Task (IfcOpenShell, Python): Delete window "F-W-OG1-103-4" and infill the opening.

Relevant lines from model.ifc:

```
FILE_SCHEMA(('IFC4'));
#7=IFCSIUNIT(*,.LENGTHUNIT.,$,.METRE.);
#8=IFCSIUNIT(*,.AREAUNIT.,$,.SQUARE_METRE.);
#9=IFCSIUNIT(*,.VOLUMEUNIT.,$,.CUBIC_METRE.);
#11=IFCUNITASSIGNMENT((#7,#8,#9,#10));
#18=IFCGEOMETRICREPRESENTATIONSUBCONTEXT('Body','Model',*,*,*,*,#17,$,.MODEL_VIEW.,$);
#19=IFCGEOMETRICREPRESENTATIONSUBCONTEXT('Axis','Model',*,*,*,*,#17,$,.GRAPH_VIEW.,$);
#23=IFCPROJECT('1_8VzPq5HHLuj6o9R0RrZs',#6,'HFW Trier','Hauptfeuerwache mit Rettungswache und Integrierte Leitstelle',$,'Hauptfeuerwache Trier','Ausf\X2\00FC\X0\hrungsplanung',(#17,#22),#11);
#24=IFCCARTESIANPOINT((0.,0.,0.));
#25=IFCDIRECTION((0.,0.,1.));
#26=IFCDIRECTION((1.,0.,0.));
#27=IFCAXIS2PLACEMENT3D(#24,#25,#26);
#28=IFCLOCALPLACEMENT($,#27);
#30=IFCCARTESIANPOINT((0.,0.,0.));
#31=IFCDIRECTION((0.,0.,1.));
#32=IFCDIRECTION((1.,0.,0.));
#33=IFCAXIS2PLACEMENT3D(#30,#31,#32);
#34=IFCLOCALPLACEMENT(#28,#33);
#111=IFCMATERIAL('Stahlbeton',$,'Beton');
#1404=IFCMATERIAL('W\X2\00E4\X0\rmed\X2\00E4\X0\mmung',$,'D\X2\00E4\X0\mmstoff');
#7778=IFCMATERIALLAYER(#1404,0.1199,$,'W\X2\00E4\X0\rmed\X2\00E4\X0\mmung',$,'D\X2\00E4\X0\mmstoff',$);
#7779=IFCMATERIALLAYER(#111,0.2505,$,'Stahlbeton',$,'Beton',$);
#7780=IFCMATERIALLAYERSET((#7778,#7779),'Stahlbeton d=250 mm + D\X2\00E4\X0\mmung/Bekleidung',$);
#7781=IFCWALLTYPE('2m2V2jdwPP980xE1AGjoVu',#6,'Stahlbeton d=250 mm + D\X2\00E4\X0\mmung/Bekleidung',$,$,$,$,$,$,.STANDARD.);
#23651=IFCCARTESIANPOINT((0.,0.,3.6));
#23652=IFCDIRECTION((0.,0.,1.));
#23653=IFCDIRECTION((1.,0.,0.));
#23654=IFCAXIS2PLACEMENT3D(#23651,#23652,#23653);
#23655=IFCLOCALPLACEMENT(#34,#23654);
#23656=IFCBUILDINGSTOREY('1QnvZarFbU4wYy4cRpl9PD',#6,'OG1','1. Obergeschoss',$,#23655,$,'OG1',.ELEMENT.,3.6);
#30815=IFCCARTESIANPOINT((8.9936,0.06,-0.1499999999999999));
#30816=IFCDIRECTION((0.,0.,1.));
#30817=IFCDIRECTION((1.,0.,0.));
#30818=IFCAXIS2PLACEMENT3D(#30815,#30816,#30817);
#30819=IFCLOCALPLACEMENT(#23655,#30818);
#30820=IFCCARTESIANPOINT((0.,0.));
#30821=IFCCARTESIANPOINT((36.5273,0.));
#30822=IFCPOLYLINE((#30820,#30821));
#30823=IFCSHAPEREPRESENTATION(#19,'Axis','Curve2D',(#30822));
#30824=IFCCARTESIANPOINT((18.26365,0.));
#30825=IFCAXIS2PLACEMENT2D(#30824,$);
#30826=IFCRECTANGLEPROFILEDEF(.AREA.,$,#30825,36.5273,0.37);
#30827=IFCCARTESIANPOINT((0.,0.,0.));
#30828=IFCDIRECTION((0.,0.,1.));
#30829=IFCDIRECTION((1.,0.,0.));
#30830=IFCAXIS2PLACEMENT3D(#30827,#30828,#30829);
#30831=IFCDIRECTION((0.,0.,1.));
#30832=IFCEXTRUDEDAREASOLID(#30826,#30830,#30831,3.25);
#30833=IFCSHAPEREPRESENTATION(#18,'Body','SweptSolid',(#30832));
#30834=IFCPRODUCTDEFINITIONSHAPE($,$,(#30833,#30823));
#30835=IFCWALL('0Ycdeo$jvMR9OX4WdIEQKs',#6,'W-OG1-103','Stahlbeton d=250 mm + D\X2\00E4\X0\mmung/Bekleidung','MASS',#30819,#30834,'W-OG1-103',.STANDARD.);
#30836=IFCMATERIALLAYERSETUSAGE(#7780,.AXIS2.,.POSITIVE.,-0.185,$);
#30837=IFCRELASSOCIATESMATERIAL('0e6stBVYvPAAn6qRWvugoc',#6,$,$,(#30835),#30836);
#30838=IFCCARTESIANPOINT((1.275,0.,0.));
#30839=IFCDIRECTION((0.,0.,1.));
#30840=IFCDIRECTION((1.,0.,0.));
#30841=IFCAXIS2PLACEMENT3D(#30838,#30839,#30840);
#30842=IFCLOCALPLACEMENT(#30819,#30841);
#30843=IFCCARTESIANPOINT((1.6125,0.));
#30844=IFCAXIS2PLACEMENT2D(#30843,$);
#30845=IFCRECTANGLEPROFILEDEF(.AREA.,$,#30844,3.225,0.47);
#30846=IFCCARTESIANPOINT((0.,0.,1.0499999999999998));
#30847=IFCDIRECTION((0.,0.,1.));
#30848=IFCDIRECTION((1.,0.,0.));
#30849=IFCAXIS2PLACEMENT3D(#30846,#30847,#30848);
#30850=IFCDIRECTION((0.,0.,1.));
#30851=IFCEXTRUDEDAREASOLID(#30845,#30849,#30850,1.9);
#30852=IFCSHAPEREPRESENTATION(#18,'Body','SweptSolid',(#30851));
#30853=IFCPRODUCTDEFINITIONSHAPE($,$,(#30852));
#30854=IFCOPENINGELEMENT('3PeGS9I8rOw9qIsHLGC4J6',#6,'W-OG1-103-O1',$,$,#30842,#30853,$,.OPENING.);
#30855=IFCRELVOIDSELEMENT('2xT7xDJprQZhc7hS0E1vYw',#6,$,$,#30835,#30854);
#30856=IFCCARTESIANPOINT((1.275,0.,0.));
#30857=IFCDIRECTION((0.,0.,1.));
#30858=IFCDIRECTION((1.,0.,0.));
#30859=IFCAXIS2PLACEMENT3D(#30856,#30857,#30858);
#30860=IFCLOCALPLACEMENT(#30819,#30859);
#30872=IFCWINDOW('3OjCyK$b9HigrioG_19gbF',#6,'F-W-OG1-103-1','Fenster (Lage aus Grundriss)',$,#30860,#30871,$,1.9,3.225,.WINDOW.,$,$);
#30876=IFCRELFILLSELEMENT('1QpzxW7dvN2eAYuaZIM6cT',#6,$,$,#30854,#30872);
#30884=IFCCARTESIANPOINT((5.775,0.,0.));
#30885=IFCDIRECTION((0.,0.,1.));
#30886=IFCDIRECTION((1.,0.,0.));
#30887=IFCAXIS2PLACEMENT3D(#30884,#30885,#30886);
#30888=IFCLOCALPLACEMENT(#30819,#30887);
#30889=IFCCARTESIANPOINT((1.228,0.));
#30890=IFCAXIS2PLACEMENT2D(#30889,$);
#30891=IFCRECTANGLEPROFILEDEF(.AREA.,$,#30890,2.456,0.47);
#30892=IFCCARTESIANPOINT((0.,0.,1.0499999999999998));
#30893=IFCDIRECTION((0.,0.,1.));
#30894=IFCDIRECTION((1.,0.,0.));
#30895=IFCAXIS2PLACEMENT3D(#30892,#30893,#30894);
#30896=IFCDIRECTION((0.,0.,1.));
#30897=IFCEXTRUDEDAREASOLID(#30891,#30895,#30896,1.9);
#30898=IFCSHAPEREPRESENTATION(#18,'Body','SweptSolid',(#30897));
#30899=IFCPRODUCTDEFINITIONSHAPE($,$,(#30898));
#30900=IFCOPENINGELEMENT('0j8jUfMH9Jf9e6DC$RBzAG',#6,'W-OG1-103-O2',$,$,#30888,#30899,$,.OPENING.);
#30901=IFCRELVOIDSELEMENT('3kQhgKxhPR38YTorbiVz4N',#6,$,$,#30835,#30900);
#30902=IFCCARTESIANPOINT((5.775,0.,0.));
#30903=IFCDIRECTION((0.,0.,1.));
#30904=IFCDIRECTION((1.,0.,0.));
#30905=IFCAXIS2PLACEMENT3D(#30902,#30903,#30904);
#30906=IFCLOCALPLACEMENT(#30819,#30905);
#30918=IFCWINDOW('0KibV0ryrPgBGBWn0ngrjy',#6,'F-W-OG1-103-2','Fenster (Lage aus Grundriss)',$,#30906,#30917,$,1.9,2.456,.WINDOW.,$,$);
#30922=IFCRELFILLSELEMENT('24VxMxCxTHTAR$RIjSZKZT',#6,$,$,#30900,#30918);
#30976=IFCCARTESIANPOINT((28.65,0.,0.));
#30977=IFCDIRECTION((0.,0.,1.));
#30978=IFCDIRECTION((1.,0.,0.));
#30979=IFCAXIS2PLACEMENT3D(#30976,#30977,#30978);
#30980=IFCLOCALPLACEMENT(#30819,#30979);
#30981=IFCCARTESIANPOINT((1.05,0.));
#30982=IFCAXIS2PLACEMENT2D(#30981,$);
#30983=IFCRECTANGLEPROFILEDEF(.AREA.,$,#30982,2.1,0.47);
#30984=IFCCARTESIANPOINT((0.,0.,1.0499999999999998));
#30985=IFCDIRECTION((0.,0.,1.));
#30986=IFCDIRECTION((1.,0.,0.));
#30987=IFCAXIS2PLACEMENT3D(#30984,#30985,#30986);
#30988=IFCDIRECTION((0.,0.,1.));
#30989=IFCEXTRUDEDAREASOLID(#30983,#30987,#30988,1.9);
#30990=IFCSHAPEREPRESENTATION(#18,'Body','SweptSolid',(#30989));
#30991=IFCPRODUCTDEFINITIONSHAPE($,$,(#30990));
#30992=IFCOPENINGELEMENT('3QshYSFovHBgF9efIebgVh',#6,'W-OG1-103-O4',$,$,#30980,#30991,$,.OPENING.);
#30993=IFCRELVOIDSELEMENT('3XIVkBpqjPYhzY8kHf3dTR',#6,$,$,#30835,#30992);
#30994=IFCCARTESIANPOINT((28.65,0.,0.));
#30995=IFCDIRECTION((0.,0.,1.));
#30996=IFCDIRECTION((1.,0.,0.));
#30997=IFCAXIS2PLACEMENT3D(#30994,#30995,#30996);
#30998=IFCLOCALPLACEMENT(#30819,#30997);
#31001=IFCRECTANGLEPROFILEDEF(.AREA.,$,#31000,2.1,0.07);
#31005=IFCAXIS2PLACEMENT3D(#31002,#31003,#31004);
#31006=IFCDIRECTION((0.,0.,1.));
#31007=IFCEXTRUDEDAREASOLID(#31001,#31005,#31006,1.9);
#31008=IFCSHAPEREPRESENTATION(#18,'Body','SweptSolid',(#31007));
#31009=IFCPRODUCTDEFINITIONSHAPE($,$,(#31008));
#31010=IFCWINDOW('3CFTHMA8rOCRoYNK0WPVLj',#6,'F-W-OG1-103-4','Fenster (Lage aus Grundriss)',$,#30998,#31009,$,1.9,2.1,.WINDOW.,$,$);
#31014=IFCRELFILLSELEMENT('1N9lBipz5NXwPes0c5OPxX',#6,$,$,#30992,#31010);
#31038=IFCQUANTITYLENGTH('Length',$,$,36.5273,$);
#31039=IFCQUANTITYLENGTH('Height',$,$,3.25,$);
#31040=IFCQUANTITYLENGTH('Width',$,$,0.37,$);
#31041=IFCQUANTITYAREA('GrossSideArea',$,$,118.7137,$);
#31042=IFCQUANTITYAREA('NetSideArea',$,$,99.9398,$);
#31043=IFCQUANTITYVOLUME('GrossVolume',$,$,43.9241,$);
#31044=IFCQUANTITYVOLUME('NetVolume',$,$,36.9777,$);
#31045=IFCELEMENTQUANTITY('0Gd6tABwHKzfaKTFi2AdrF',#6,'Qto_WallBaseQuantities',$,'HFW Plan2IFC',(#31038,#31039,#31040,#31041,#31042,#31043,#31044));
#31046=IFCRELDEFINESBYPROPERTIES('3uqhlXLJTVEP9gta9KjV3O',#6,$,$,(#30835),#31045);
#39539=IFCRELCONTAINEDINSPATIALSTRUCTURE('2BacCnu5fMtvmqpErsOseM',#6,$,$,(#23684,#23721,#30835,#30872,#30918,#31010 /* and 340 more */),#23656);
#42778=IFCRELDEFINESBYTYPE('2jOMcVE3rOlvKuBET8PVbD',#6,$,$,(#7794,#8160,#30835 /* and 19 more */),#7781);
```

```python
import ifcopenshell
import ifcopenshell.api.feature
import ifcopenshell.api.pset
import ifcopenshell.api.root
import ifcopenshell.geom
import ifcopenshell.util.element
import ifcopenshell.util.shape
import ifcopenshell.util.unit

model = ifcopenshell.open("model.ifc")
area_scale = ifcopenshell.util.unit.calculate_unit_scale(model, "AREAUNIT")
volume_scale = ifcopenshell.util.unit.calculate_unit_scale(model, "VOLUMEUNIT")
settings = ifcopenshell.geom.settings()


def volume(element):
    """Net volume in cubic metres, openings subtracted."""
    shape = ifcopenshell.geom.create_shape(settings, element)
    return ifcopenshell.util.shape.get_volume(shape.geometry)


window = model.by_id(31010)
opening = window.FillsVoids[0].RelatingOpeningElement
wall = opening.VoidsElements[0].RelatingBuildingElement
before = volume(wall)

ifcopenshell.api.root.remove_product(model, product=window)
ifcopenshell.api.feature.remove_feature(model, feature=opening)

after = volume(wall)
thickness = 0.37  # wall thickness in metres

# Update the wall's stored quantities.
qto = model.by_id(ifcopenshell.util.element.get_pset(wall, "Qto_WallBaseQuantities", should_inherit=False)["id"])
ifcopenshell.api.pset.edit_qto(model, qto=qto, properties={
    "NetSideArea": after / thickness / area_scale,
    "NetVolume": after / volume_scale,
})

print(f"wall volume {before:.3f} -> {after:.3f} m3")

model.write("model_updated.ifc")
```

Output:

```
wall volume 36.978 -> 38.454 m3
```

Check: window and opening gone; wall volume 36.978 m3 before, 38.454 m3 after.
